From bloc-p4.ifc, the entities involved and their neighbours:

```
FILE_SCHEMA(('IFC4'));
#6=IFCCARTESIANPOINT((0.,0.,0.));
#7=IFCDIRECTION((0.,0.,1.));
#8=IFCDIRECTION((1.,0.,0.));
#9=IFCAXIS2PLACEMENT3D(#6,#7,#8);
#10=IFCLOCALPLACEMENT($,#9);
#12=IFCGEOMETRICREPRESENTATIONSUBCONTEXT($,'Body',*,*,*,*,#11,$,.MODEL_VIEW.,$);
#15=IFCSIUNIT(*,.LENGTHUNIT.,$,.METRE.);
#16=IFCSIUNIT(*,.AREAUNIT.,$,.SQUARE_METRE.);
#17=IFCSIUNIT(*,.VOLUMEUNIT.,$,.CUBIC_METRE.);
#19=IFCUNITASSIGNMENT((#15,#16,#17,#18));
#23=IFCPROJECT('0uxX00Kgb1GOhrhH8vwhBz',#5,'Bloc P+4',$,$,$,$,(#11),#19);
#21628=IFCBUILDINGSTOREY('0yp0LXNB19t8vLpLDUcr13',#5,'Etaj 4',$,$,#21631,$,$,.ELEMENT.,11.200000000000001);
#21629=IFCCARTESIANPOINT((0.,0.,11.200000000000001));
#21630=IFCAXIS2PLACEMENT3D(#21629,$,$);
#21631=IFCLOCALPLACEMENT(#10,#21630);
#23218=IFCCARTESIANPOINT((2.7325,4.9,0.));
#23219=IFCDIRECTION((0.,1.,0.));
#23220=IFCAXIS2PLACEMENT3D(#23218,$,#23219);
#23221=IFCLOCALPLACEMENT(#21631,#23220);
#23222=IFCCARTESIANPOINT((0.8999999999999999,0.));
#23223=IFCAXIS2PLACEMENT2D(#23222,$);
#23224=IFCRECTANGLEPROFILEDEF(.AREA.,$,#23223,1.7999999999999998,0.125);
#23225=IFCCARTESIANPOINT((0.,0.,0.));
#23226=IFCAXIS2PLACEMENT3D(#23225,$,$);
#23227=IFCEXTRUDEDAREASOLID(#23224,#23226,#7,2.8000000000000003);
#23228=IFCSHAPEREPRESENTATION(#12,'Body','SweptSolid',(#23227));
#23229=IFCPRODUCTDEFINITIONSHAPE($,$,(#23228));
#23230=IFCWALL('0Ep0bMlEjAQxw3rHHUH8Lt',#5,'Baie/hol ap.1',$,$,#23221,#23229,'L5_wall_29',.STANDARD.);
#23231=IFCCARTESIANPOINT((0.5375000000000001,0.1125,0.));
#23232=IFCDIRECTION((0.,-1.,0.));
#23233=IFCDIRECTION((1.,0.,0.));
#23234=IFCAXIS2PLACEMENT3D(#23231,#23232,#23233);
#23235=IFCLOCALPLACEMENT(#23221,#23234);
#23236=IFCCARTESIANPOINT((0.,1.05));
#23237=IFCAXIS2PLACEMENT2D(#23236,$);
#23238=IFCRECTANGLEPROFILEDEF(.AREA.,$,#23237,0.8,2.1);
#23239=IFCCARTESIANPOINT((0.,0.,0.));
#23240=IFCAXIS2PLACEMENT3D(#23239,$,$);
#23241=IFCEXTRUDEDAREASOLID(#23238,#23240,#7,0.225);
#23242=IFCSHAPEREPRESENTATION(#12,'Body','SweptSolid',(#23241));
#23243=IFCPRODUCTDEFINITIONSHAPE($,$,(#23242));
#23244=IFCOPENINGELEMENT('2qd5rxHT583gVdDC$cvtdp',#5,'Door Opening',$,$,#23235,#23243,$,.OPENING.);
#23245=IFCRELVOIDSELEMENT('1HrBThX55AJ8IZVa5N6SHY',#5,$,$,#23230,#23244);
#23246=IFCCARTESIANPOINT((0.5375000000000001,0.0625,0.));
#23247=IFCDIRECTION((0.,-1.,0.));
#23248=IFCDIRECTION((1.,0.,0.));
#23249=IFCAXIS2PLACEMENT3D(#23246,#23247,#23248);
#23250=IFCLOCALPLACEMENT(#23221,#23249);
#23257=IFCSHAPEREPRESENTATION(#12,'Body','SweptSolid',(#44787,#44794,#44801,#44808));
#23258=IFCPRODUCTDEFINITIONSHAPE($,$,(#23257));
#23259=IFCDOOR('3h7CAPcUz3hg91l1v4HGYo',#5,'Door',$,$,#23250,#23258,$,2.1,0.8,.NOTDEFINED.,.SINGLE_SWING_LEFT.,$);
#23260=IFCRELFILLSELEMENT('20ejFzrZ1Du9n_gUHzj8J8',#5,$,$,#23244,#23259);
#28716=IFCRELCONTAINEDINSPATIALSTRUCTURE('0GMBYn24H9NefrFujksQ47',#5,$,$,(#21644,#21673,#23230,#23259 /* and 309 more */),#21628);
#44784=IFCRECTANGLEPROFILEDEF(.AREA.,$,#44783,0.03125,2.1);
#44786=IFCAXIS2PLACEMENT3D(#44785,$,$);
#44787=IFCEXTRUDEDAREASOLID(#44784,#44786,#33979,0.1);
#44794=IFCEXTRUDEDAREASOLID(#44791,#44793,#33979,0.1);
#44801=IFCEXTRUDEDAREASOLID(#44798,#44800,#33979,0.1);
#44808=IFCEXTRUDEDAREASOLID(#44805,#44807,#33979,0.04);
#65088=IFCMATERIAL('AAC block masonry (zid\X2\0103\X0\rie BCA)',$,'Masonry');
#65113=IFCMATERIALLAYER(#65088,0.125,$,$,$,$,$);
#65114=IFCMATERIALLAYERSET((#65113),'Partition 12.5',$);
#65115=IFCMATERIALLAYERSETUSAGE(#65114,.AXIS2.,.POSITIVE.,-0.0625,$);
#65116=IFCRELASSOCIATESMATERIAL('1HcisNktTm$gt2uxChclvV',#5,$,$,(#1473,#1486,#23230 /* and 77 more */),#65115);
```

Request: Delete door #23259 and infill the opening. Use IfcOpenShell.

```python
import ifcopenshell
import ifcopenshell.api.feature
import ifcopenshell.api.root
import ifcopenshell.geom
import ifcopenshell.util.shape

model = ifcopenshell.open("bloc-p4.ifc")
settings = ifcopenshell.geom.settings()


def volume(element):
    """Net volume in cubic metres, openings subtracted."""
    shape = ifcopenshell.geom.create_shape(settings, element)
    return ifcopenshell.util.shape.get_volume(shape.geometry)


door = model.by_id(23259)
opening = door.FillsVoids[0].RelatingOpeningElement
wall = opening.VoidsElements[0].RelatingBuildingElement
before = volume(wall)

ifcopenshell.api.root.remove_product(model, product=door)
ifcopenshell.api.feature.remove_feature(model, feature=opening)

after = volume(wall)

print(f"wall volume {before:.3f} -> {after:.3f} m3")

model.write("bloc-p4_v2.ifc")
```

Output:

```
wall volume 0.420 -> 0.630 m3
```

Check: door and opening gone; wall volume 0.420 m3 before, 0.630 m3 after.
